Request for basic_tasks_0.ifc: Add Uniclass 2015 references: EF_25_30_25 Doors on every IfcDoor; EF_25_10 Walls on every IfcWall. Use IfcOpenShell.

First a look at what the model holds.

```python
import ifcopenshell

model = ifcopenshell.open("basic_tasks_0.ifc")
print(model.schema)
print("classifications:", [c.Name for c in model.by_type("IfcClassification")])
for ifc_class in ("IfcDoor", "IfcRoof", "IfcStair", "IfcWall", "IfcWindow"):
    print(ifc_class, len(model.by_type(ifc_class)))
```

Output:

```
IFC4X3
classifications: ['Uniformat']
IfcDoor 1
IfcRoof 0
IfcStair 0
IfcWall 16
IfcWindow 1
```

```python
import ifcopenshell
import ifcopenshell.api.classification

model = ifcopenshell.open("basic_tasks_0.ifc")

system = ifcopenshell.api.classification.add_classification(model, classification="Uniclass 2015")

codes = {
    "IfcDoor": ("EF_25_30_25", "Doors"),
    "IfcWall": ("EF_25_10", "Walls"),
}
for ifc_class, (code, name) in codes.items():
    products = model.by_type(ifc_class)
    ifcopenshell.api.classification.add_reference(
        model, products=products, classification=system, identification=code, name=name
    )
    print(code, len(products))

model.write("basic_tasks_0_rev.ifc")
```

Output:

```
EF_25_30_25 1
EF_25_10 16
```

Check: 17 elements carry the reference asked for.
